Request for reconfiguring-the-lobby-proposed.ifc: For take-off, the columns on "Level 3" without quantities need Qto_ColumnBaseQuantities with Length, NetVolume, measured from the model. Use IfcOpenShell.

First a look at what the model holds.

```python
import ifcopenshell
import ifcopenshell.util.element
import ifcopenshell.util.unit

model = ifcopenshell.open("reconfiguring-the-lobby-proposed.ifc")
print(model.schema)
for unit_type in ("LENGTHUNIT", "AREAUNIT", "VOLUMEUNIT"):
    print(unit_type, ifcopenshell.util.unit.calculate_unit_scale(model, unit_type))
storey = next(s for s in model.by_type("IfcBuildingStorey") if s.Name == "Level 3")
columns = [e for e in ifcopenshell.util.element.get_decomposition(storey) if e.is_a("IfcColumn")]
for e in sorted(columns, key=lambda e: e.id()):
    print(e.id(), e.is_a(), e.Name, list(ifcopenshell.util.element.get_psets(e, qtos_only=True)), sep=" | ")
```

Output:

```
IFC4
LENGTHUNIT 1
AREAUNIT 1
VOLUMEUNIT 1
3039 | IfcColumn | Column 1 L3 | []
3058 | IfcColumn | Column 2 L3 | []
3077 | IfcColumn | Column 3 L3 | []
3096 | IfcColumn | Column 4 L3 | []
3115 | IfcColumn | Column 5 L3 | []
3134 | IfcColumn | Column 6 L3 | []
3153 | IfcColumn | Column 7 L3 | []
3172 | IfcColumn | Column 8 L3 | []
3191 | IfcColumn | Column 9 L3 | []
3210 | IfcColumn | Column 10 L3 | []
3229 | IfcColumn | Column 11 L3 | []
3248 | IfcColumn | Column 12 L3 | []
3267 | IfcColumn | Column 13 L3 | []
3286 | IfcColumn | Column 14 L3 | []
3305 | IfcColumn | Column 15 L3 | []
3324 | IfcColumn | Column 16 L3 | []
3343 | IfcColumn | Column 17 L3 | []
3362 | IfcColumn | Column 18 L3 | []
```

```python
import ifcopenshell
import ifcopenshell.api.pset
import ifcopenshell.geom
import ifcopenshell.util.element
import ifcopenshell.util.shape
import ifcopenshell.util.unit

model = ifcopenshell.open("reconfiguring-the-lobby-proposed.ifc")
unit_scale = ifcopenshell.util.unit.calculate_unit_scale(model)
volume_scale = ifcopenshell.util.unit.calculate_unit_scale(model, "VOLUMEUNIT")
settings = ifcopenshell.geom.settings()

storey = next(s for s in model.by_type("IfcBuildingStorey") if s.Name == "Level 3")
columns = [e for e in ifcopenshell.util.element.get_decomposition(storey) if e.is_a("IfcColumn")]

for e in sorted(columns, key=lambda e: e.id()):
    if ifcopenshell.util.element.get_psets(e, qtos_only=True, should_inherit=False):
        continue
    # Geometry comes back in metres, in the element's own axes.
    shape = ifcopenshell.geom.create_shape(settings, e)
    values = {
        "Length": ifcopenshell.util.shape.get_z(shape.geometry) / unit_scale,
        "NetVolume": ifcopenshell.util.shape.get_volume(shape.geometry) / volume_scale,
    }
    qto = ifcopenshell.api.pset.add_qto(model, product=e, name="Qto_ColumnBaseQuantities")
    ifcopenshell.api.pset.edit_qto(model, qto=qto, properties=values)
    print(e.id(), {k: round(v, 3) for k, v in values.items()})

model.write("reconfiguring-the-lobby-proposed_edited.ifc")
```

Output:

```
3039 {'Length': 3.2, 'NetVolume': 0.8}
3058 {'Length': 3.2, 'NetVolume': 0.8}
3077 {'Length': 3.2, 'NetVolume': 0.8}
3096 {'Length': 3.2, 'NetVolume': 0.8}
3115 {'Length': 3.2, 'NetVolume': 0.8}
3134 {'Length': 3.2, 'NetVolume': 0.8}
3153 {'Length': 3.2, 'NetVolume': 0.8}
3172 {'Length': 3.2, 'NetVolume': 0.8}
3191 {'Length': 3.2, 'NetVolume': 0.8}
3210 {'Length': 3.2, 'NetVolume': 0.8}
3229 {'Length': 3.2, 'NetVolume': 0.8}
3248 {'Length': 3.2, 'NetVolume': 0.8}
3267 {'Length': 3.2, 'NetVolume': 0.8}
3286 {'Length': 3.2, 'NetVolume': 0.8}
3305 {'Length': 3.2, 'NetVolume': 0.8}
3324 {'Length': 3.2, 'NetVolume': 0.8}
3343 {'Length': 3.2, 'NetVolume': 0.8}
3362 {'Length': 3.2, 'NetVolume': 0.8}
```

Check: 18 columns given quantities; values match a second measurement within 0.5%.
